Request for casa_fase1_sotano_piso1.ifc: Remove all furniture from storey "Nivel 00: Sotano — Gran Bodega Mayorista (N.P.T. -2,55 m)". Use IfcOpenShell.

First a look at what the model holds.

```python
import ifcopenshell
import ifcopenshell.util.element

model = ifcopenshell.open("casa_fase1_sotano_piso1.ifc")
print(model.schema)
storey = next(s for s in model.by_type("IfcBuildingStorey") if s.Name == "Nivel 00: Sotano — Gran Bodega Mayorista (N.P.T. -2,55 m)")
furniture = [e for e in ifcopenshell.util.element.get_decomposition(storey) if e.is_a("IfcFurnishingElement")]
seen = {}
for e in furniture:
    element_type = ifcopenshell.util.element.get_type(e)
    name = element_type.Name if element_type not in (None, e) else None
    seen[name] = seen.get(name, 0) + 1
for name, count in sorted(seen.items(), key=str):
    print(count, "x", name)
```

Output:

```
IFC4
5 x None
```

```python
import ifcopenshell
import ifcopenshell.api.root
import ifcopenshell.util.element

model = ifcopenshell.open("casa_fase1_sotano_piso1.ifc")

storey = next(s for s in model.by_type("IfcBuildingStorey") if s.Name == "Nivel 00: Sotano — Gran Bodega Mayorista (N.P.T. -2,55 m)")
furniture = [e for e in ifcopenshell.util.element.get_decomposition(storey) if e.is_a("IfcFurnishingElement")]

for e in furniture:
    ifcopenshell.api.root.remove_product(model, product=e)
print(len(furniture), "removed")

model.write("casa_fase1_sotano_piso1-out.ifc")
```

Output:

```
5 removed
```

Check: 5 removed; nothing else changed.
